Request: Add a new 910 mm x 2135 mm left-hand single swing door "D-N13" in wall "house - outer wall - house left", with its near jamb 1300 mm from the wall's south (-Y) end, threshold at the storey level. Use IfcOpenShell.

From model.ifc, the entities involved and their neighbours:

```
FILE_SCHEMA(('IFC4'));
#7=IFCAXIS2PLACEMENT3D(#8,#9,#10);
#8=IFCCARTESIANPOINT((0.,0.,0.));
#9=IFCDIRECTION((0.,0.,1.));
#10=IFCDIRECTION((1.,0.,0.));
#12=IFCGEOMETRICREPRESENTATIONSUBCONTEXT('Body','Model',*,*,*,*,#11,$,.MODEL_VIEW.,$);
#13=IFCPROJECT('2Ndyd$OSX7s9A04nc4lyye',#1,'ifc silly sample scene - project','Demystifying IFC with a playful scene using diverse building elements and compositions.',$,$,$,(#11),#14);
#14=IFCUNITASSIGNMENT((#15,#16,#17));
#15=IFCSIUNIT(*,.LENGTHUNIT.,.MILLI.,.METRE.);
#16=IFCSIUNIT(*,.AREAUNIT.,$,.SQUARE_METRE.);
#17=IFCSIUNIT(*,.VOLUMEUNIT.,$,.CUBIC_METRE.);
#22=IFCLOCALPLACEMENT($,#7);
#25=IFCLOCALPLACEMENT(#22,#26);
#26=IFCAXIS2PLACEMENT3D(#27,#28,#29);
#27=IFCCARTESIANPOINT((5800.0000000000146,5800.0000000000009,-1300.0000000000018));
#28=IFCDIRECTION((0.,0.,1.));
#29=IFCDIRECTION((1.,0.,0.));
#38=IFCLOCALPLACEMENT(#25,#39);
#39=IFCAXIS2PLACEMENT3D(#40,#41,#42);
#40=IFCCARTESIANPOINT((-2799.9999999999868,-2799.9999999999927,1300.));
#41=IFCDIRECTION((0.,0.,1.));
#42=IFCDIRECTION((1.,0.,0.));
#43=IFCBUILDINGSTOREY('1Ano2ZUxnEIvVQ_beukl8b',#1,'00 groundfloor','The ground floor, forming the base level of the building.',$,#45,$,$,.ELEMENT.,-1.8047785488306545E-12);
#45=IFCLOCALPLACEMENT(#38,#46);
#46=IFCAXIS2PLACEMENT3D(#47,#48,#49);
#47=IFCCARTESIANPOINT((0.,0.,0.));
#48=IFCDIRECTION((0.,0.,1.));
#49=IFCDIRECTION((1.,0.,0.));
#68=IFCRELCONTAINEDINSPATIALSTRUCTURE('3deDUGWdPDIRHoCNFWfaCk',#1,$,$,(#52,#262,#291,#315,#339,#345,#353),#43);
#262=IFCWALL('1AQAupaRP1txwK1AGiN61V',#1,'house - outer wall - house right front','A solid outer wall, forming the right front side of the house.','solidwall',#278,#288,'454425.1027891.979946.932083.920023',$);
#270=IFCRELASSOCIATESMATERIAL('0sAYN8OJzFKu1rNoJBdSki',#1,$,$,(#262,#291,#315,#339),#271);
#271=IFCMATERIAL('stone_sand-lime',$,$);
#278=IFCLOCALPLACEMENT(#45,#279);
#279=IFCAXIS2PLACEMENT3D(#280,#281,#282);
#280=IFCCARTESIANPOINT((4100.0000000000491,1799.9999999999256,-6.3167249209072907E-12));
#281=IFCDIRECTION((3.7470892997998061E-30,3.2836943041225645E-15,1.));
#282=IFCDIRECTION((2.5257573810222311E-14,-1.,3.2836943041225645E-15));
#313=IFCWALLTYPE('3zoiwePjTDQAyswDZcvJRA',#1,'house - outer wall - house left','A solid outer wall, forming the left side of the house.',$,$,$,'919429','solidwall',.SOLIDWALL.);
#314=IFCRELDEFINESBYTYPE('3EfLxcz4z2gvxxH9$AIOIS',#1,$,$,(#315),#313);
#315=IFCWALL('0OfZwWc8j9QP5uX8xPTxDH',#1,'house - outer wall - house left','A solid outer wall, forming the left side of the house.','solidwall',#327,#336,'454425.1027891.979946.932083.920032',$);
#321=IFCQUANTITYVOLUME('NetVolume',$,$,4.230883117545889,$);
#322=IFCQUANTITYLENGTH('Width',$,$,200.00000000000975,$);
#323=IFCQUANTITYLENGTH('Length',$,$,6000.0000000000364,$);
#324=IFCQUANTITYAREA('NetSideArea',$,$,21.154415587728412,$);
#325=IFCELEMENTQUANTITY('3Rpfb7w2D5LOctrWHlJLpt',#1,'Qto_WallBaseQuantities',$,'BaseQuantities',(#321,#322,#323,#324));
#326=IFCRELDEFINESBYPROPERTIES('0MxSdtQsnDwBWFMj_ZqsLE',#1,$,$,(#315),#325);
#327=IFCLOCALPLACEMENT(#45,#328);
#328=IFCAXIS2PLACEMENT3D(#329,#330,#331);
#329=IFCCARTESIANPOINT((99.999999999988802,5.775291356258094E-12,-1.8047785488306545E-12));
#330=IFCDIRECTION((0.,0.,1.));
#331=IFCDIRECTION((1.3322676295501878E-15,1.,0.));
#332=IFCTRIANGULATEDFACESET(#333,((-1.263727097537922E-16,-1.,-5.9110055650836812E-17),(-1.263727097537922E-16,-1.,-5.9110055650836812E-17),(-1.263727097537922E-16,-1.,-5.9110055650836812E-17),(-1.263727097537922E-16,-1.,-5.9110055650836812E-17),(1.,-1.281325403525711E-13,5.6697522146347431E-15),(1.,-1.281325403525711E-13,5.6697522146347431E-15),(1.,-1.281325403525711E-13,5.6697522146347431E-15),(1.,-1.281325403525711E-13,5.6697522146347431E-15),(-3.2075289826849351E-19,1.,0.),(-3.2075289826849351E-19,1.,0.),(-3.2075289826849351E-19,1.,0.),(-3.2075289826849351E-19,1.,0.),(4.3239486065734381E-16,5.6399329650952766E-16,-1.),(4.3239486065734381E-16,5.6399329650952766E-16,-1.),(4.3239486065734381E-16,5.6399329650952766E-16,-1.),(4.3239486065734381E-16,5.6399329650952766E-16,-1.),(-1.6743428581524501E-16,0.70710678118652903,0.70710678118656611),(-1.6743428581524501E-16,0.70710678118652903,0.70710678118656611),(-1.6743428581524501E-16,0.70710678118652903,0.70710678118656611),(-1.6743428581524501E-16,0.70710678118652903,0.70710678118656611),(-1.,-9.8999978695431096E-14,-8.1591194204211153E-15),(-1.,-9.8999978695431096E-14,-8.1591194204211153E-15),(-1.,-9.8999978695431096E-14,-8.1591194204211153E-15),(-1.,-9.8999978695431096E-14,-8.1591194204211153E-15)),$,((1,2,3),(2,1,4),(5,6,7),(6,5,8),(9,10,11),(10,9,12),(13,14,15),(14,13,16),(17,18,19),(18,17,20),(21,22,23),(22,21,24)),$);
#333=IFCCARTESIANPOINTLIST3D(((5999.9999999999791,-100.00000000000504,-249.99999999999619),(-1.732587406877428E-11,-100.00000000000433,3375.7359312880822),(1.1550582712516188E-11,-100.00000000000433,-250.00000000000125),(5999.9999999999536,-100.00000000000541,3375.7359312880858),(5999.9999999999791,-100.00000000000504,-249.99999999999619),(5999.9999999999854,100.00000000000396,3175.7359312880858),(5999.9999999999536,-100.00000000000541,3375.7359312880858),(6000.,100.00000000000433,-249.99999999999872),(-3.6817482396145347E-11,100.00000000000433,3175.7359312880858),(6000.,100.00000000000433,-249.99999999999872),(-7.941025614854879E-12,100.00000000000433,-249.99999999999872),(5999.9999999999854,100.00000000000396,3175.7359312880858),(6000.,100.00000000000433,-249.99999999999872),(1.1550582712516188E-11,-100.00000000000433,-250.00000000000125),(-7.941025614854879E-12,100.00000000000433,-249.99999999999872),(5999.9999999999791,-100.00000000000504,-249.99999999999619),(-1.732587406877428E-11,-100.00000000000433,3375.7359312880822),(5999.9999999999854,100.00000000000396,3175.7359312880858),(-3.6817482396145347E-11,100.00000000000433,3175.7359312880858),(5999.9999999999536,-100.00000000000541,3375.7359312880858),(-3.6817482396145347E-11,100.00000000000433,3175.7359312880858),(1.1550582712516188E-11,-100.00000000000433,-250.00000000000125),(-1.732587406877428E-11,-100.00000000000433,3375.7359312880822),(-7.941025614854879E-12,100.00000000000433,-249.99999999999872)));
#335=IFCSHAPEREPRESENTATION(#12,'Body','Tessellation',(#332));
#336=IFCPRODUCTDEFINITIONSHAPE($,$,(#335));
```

```python
import numpy as np
import ifcopenshell
import ifcopenshell.api.feature
import ifcopenshell.api.geometry
import ifcopenshell.api.pset
import ifcopenshell.api.root
import ifcopenshell.api.spatial
import ifcopenshell.geom
import ifcopenshell.util.element
import ifcopenshell.util.placement
import ifcopenshell.util.representation
import ifcopenshell.util.shape
import ifcopenshell.util.unit

model = ifcopenshell.open("model.ifc")
unit_scale = ifcopenshell.util.unit.calculate_unit_scale(model)
area_scale = ifcopenshell.util.unit.calculate_unit_scale(model, "AREAUNIT")
volume_scale = ifcopenshell.util.unit.calculate_unit_scale(model, "VOLUMEUNIT")
settings = ifcopenshell.geom.settings()


def volume(element):
    """Net volume in cubic metres, openings subtracted."""
    shape = ifcopenshell.geom.create_shape(settings, element)
    return ifcopenshell.util.shape.get_volume(shape.geometry)


wall = model.by_guid("0OfZwWc8j9QP5uX8xPTxDH")
storey = ifcopenshell.util.element.get_container(wall, ifc_class="IfcBuildingStorey")
context = ifcopenshell.util.representation.get_context(model, "Model", "Body", "MODEL_VIEW")
before = volume(wall)

width, height, from_end, sill = 0.91, 2.135, 1.3, 0.0  # metres

# The wall runs along its own X axis, and the end named is its -X end.
wall_shape = ifcopenshell.geom.create_shape(settings, wall)
x, y, z = ifcopenshell.util.shape.get_vertices(wall_shape.geometry).T
start = x.min() + from_end
face, thickness = float(y.min()), float(y.max() - y.min())
wall_matrix = ifcopenshell.util.placement.get_local_placement(wall.ObjectPlacement)
level = ifcopenshell.util.placement.get_local_placement(storey.ObjectPlacement)[2, 3]


def in_wall(x, y):
    """Placement at x, y metres in the wall's axes, at sill height."""
    matrix = wall_matrix.copy()
    matrix[:, 3] = wall_matrix @ np.array([x / unit_scale, y / unit_scale, 0.0, 1.0])
    matrix[2, 3] = level + sill / unit_scale
    return matrix


# Opening: a box that overshoots both wall faces by 50 mm.
opening = ifcopenshell.api.root.create_entity(model, ifc_class="IfcOpeningElement", predefined_type="OPENING")
box = ifcopenshell.api.geometry.add_wall_representation(
    model, context=context, length=width, height=height, thickness=thickness + 0.1
)
ifcopenshell.api.geometry.assign_representation(model, product=opening, representation=box)
ifcopenshell.api.geometry.edit_object_placement(model, product=opening, matrix=in_wall(start, face - 0.05), is_si=False)
ifcopenshell.api.feature.add_feature(model, feature=opening, element=wall)

door = ifcopenshell.api.root.create_entity(model, ifc_class="IfcDoor", name="D-N13", predefined_type="DOOR")
door.OverallWidth, door.OverallHeight = width / unit_scale, height / unit_scale
door.OperationType = "SINGLE_SWING_LEFT"
body = ifcopenshell.api.geometry.add_door_representation(
    model,
    context=context,
    overall_width=door.OverallWidth,
    overall_height=door.OverallHeight,
    operation_type="SINGLE_SWING_LEFT",
    lining_properties={"LiningDepth": thickness / unit_scale, "ThresholdDepth": thickness / unit_scale},
)
ifcopenshell.api.geometry.assign_representation(model, product=door, representation=body)
ifcopenshell.api.spatial.assign_container(model, products=[door], relating_structure=storey)
ifcopenshell.api.feature.add_filling(model, opening=opening, element=door)

# The lining spans the wall, so the door starts at the wall face.
ifcopenshell.api.geometry.edit_object_placement(model, product=door, matrix=in_wall(start, face), is_si=False)

after = volume(wall)

# Update the wall's stored quantities.
qto = model.by_id(ifcopenshell.util.element.get_pset(wall, "Qto_WallBaseQuantities", should_inherit=False)["id"])
ifcopenshell.api.pset.edit_qto(model, qto=qto, properties={
    "NetVolume": after / volume_scale,
    "NetSideArea": after / thickness / area_scale,
})

print(f"wall volume {before:.3f} -> {after:.3f} m3")

model.write("model_rev.ifc")
```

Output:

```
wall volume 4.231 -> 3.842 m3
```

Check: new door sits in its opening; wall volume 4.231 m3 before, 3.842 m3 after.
